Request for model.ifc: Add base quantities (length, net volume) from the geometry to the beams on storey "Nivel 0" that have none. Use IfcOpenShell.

First a look at what the model holds.

```python
import ifcopenshell
import ifcopenshell.util.element
import ifcopenshell.util.unit

model = ifcopenshell.open("model.ifc")
print(model.schema)
for unit_type in ("LENGTHUNIT", "AREAUNIT", "VOLUMEUNIT"):
    print(unit_type, ifcopenshell.util.unit.calculate_unit_scale(model, unit_type))
storey = next(s for s in model.by_type("IfcBuildingStorey") if s.Name == "Nivel 0")
beams = [e for e in ifcopenshell.util.element.get_decomposition(storey) if e.is_a("IfcBeam")]
for e in sorted(beams, key=lambda e: e.id()):
    print(e.id(), e.is_a(), e.Name, list(ifcopenshell.util.element.get_psets(e, qtos_only=True)), sep=" | ")
```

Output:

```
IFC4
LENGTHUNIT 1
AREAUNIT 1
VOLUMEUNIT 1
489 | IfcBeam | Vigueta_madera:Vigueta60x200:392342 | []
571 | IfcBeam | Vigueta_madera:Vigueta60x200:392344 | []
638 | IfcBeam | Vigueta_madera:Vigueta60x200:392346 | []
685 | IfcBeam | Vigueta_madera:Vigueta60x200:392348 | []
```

```python
import ifcopenshell
import ifcopenshell.api.pset
import ifcopenshell.geom
import ifcopenshell.util.element
import ifcopenshell.util.shape
import ifcopenshell.util.unit

model = ifcopenshell.open("model.ifc")
unit_scale = ifcopenshell.util.unit.calculate_unit_scale(model)
volume_scale = ifcopenshell.util.unit.calculate_unit_scale(model, "VOLUMEUNIT")
settings = ifcopenshell.geom.settings()

storey = next(s for s in model.by_type("IfcBuildingStorey") if s.Name == "Nivel 0")
beams = [e for e in ifcopenshell.util.element.get_decomposition(storey) if e.is_a("IfcBeam")]

for e in sorted(beams, key=lambda e: e.id()):
    if ifcopenshell.util.element.get_psets(e, qtos_only=True, should_inherit=False):
        continue
    # Geometry comes back in metres, in the element's own axes.
    shape = ifcopenshell.geom.create_shape(settings, e)
    values = {
        "Length": ifcopenshell.util.shape.get_max_xyz(shape.geometry) / unit_scale,
        "NetVolume": ifcopenshell.util.shape.get_volume(shape.geometry) / volume_scale,
    }
    qto = ifcopenshell.api.pset.add_qto(model, product=e, name="Qto_BeamBaseQuantities")
    ifcopenshell.api.pset.edit_qto(model, qto=qto, properties=values)
    print(e.id(), {k: round(v, 3) for k, v in values.items()})

model.write("model_v2.ifc")
```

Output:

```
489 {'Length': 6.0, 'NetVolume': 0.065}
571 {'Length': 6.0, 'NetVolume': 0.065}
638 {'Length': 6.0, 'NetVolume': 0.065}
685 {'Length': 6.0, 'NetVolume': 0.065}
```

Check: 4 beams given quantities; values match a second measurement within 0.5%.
